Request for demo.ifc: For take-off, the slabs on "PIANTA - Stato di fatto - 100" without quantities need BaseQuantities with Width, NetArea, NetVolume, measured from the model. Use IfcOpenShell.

First a look at what the model holds.

```python
import ifcopenshell
import ifcopenshell.util.element
import ifcopenshell.util.unit

model = ifcopenshell.open("demo.ifc")
print(model.schema)
for unit_type in ("LENGTHUNIT", "AREAUNIT", "VOLUMEUNIT"):
    print(unit_type, ifcopenshell.util.unit.calculate_unit_scale(model, unit_type))
storey = next(s for s in model.by_type("IfcBuildingStorey") if s.Name == "PIANTA - Stato di fatto - 100")
slabs = [e for e in ifcopenshell.util.element.get_decomposition(storey) if e.is_a("IfcSlab")]
for e in sorted(slabs, key=lambda e: e.id()):
    print(e.id(), e.is_a(), e.Name, list(ifcopenshell.util.element.get_psets(e, qtos_only=True)), sep=" | ")
```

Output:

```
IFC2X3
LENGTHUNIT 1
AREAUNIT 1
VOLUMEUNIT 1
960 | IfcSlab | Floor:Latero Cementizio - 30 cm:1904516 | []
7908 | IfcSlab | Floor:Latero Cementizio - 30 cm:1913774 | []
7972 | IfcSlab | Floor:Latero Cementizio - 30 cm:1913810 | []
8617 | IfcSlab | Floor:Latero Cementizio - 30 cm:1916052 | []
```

```python
import ifcopenshell
import ifcopenshell.api.pset
import ifcopenshell.geom
import ifcopenshell.util.element
import ifcopenshell.util.shape
import ifcopenshell.util.unit

model = ifcopenshell.open("demo.ifc")
unit_scale = ifcopenshell.util.unit.calculate_unit_scale(model)
area_scale = ifcopenshell.util.unit.calculate_unit_scale(model, "AREAUNIT")
volume_scale = ifcopenshell.util.unit.calculate_unit_scale(model, "VOLUMEUNIT")
settings = ifcopenshell.geom.settings()

storey = next(s for s in model.by_type("IfcBuildingStorey") if s.Name == "PIANTA - Stato di fatto - 100")
slabs = [e for e in ifcopenshell.util.element.get_decomposition(storey) if e.is_a("IfcSlab")]

for e in sorted(slabs, key=lambda e: e.id()):
    if ifcopenshell.util.element.get_psets(e, qtos_only=True, should_inherit=False):
        continue
    # Geometry comes back in metres, in the element's own axes.
    shape = ifcopenshell.geom.create_shape(settings, e)
    values = {
        "Width": ifcopenshell.util.shape.get_z(shape.geometry) / unit_scale,
        "NetArea": ifcopenshell.util.shape.get_footprint_area(shape.geometry) / area_scale,
        "NetVolume": ifcopenshell.util.shape.get_volume(shape.geometry) / volume_scale,
    }
    qto = ifcopenshell.api.pset.add_qto(model, product=e, name="BaseQuantities")
    ifcopenshell.api.pset.edit_qto(model, qto=qto, properties=values)
    print(e.id(), {k: round(v, 3) for k, v in values.items()})

model.write("demo_rev.ifc")
```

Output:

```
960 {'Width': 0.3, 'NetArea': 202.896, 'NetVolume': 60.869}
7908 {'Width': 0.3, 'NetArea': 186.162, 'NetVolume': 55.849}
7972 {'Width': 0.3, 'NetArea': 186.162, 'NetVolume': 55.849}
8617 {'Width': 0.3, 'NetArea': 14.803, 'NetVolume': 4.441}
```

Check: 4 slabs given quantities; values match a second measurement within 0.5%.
